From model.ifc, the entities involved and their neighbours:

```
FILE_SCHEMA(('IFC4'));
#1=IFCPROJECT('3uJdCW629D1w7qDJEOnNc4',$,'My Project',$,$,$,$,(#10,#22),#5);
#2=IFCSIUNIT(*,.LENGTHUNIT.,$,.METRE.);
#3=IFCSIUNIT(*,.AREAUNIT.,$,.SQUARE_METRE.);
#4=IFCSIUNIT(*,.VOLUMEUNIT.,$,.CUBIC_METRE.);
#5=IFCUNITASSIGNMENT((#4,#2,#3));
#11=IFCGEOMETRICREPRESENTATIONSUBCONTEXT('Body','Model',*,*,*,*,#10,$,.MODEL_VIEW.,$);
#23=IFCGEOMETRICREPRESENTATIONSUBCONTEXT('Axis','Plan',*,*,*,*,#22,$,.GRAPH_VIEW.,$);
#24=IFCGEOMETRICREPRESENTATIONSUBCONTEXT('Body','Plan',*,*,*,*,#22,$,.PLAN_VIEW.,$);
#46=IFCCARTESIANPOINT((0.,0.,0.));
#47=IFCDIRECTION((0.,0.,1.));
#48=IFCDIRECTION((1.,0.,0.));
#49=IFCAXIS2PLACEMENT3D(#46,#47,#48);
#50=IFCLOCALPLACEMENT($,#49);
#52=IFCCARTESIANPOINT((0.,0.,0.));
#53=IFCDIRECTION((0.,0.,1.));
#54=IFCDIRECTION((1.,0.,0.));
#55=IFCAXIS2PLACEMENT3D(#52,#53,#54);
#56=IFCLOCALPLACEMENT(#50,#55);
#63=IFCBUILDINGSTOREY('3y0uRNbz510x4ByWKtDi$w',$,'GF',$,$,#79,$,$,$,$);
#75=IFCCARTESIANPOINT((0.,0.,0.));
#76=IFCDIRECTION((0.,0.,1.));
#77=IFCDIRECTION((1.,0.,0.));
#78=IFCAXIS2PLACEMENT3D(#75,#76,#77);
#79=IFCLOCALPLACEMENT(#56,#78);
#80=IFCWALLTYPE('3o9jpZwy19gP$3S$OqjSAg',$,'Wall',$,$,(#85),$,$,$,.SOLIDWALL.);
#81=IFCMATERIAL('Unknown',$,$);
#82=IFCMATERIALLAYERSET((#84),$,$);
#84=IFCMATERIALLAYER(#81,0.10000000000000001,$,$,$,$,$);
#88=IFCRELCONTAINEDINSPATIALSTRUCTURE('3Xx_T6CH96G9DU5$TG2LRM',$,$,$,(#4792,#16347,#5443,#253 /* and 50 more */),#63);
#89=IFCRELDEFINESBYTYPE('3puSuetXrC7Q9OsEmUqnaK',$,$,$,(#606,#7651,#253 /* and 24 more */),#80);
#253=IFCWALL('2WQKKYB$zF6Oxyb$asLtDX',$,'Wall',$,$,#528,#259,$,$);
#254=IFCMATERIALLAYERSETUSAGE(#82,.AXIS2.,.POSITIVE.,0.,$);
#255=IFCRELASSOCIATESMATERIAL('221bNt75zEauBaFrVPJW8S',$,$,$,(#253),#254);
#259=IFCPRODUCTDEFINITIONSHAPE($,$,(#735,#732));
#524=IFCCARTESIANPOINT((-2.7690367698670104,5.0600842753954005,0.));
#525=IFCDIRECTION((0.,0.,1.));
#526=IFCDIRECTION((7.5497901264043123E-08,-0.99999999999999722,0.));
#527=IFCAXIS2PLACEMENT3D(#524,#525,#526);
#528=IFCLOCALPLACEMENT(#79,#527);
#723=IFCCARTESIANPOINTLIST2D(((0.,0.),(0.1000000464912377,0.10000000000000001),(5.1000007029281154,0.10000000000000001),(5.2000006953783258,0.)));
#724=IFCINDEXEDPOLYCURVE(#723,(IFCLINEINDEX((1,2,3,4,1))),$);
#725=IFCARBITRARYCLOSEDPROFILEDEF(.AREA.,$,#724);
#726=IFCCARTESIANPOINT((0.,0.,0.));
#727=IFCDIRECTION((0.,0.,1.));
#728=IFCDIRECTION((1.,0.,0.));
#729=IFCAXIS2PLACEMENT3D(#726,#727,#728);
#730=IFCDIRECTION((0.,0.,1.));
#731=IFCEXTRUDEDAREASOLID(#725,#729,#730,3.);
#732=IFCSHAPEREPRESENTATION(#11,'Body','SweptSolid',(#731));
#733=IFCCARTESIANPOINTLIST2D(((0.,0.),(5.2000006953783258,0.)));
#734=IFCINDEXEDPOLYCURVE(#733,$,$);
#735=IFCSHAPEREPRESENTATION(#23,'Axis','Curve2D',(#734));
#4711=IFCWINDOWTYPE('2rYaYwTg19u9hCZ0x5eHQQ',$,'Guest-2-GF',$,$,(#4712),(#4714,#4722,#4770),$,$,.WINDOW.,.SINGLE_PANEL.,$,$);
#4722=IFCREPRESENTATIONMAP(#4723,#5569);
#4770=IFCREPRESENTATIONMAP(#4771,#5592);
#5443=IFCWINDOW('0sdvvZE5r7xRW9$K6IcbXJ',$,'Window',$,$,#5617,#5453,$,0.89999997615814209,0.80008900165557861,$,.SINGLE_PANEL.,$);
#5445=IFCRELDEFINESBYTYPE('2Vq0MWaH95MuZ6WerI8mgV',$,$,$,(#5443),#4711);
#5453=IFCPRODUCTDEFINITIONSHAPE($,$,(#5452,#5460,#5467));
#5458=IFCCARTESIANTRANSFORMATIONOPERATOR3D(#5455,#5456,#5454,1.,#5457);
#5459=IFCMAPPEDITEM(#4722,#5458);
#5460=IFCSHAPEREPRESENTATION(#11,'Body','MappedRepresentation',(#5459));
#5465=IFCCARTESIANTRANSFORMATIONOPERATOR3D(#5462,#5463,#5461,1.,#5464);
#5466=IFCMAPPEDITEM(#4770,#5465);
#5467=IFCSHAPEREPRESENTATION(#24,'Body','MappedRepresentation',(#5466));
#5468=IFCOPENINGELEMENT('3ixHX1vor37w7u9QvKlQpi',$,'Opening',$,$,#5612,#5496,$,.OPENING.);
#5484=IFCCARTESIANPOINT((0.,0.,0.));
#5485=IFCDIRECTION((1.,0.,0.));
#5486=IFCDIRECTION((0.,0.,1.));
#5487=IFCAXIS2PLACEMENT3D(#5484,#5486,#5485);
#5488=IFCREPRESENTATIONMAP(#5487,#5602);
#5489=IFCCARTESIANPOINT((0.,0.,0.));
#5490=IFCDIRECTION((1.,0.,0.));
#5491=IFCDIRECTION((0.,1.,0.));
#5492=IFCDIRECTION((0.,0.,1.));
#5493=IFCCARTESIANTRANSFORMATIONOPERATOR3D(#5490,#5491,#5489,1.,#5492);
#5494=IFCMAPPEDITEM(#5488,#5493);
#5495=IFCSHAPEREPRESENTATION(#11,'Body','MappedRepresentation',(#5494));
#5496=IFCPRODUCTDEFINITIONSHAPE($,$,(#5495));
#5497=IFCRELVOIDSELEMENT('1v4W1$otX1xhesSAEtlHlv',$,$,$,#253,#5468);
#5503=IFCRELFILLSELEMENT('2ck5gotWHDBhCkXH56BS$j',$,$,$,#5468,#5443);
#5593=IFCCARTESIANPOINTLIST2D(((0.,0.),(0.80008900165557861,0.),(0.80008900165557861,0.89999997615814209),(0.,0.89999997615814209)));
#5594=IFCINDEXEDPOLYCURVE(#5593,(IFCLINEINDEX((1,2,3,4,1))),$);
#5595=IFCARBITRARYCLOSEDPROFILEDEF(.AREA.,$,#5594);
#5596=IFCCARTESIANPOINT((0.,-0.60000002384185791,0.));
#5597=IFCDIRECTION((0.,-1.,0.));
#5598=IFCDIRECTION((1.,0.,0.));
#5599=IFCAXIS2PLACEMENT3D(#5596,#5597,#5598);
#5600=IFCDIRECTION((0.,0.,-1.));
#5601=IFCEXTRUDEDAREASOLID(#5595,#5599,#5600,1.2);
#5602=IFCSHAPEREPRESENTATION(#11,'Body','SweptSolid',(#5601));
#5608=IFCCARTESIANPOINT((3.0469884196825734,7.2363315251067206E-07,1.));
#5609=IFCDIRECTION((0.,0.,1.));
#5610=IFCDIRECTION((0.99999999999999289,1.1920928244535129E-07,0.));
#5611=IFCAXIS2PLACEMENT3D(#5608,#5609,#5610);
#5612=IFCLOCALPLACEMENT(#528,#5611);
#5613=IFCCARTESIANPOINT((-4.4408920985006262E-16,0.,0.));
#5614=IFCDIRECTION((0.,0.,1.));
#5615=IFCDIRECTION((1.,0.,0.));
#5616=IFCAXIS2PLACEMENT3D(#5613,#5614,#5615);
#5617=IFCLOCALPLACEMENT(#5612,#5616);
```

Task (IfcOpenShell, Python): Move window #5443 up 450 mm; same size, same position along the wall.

```python
import numpy as np
import ifcopenshell
import ifcopenshell.api.geometry
import ifcopenshell.util.placement
import ifcopenshell.util.unit

model = ifcopenshell.open("model.ifc")
unit_scale = ifcopenshell.util.unit.calculate_unit_scale(model)

window = model.by_guid("0sdvvZE5r7xRW9$K6IcbXJ")
opening = window.FillsVoids[0].RelatingOpeningElement
dz = 0.45

shift = np.array([0.0, 0.0, dz])
# The window is placed relative to its opening, so it follows when the opening moves.
matrix = ifcopenshell.util.placement.get_local_placement(opening.ObjectPlacement)
matrix[:3, 3] += shift
ifcopenshell.api.geometry.edit_object_placement(
    model, product=opening, matrix=matrix, is_si=False, should_transform_children=True
)

print(f"moved by {dz * unit_scale:+.3f} m")

model.write("model_v2.ifc")
```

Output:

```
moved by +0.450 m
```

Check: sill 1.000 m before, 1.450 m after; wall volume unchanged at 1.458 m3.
